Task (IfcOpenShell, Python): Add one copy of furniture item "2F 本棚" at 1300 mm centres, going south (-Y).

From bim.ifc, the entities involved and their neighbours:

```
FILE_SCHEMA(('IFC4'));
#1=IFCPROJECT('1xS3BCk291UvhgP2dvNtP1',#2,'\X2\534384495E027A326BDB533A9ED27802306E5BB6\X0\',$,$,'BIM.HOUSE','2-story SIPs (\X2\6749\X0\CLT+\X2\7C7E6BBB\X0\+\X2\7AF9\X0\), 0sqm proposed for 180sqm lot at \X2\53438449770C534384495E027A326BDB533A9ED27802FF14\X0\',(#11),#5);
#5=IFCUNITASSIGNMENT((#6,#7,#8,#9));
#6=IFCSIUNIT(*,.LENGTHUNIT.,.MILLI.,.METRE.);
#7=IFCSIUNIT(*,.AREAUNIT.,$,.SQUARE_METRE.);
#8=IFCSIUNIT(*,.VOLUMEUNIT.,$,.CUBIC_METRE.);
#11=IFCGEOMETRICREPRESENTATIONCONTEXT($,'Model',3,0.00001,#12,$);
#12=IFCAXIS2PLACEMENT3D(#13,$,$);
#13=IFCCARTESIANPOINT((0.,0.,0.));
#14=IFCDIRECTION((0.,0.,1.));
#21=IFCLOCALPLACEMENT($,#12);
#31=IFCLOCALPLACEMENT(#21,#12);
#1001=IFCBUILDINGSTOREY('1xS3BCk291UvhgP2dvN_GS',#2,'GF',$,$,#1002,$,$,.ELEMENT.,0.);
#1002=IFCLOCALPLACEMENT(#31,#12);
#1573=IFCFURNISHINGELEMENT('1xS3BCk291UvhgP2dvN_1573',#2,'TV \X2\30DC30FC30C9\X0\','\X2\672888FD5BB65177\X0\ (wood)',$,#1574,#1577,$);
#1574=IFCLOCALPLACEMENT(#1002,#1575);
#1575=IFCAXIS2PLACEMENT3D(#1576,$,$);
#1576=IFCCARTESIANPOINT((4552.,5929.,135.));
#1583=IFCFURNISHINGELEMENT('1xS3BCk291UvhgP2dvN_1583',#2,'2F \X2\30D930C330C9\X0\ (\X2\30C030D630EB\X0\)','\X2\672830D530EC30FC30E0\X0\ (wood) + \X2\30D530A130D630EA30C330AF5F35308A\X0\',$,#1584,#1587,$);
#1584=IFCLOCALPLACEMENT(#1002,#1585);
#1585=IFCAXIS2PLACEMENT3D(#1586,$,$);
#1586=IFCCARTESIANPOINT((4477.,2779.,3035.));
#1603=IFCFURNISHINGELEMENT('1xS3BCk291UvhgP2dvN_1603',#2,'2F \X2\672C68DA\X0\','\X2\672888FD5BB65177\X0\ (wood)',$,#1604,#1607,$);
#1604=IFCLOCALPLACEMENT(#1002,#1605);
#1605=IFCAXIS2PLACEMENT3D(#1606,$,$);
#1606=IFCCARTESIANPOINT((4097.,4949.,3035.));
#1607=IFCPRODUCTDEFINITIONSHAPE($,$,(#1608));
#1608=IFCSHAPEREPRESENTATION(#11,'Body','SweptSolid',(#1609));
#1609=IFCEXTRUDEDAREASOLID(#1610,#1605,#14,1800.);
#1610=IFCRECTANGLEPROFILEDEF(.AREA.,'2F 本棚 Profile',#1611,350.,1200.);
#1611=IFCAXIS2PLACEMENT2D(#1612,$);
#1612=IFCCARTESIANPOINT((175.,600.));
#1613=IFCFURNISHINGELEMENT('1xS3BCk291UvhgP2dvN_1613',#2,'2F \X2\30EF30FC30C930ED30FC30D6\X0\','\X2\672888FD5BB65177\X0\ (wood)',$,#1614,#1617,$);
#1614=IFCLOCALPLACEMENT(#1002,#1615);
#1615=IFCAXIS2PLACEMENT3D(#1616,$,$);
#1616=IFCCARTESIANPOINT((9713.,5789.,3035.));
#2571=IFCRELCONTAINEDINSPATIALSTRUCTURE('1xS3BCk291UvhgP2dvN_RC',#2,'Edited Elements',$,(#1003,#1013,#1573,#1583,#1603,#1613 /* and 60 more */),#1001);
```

```python
import numpy as np
import ifcopenshell
import ifcopenshell.api.geometry
import ifcopenshell.api.root
import ifcopenshell.util.element
import ifcopenshell.util.placement
import ifcopenshell.util.unit

model = ifcopenshell.open("bim.ifc")
unit_scale = ifcopenshell.util.unit.calculate_unit_scale(model)


def reuse_history(source, copy):
    """copy_class also copies each property set's owner history, people and application; keep the originals."""
    for rel in copy.IsDefinedBy:
        if rel.is_a("IfcRelDefinesByProperties") and (history := rel.RelatingPropertyDefinition.OwnerHistory):
            rel.RelatingPropertyDefinition.OwnerHistory = source.OwnerHistory
            ifcopenshell.util.element.remove_deep2(model, history)


source = model.by_guid("1xS3BCk291UvhgP2dvN_1603")
base = ifcopenshell.util.placement.get_local_placement(source.ObjectPlacement)
step = np.array([0.0, -1.0, 0.0]) * 1.3 / unit_scale

for i in range(1, 2):
    copy = ifcopenshell.api.root.copy_class(model, product=source)
    copy.Representation = ifcopenshell.util.element.copy_deep(
        model, source.Representation, exclude=["IfcGeometricRepresentationContext", "IfcRepresentationMap"]
    )
    reuse_history(source, copy)
    matrix = base.copy()
    matrix[:3, 3] += i * step
    print("added at", matrix[:3, 3].round(3) + 0.0)
    ifcopenshell.api.geometry.edit_object_placement(model, product=copy, matrix=matrix, is_si=False)

model.write("bim_edited.ifc")
```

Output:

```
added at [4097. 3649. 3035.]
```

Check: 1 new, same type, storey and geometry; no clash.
